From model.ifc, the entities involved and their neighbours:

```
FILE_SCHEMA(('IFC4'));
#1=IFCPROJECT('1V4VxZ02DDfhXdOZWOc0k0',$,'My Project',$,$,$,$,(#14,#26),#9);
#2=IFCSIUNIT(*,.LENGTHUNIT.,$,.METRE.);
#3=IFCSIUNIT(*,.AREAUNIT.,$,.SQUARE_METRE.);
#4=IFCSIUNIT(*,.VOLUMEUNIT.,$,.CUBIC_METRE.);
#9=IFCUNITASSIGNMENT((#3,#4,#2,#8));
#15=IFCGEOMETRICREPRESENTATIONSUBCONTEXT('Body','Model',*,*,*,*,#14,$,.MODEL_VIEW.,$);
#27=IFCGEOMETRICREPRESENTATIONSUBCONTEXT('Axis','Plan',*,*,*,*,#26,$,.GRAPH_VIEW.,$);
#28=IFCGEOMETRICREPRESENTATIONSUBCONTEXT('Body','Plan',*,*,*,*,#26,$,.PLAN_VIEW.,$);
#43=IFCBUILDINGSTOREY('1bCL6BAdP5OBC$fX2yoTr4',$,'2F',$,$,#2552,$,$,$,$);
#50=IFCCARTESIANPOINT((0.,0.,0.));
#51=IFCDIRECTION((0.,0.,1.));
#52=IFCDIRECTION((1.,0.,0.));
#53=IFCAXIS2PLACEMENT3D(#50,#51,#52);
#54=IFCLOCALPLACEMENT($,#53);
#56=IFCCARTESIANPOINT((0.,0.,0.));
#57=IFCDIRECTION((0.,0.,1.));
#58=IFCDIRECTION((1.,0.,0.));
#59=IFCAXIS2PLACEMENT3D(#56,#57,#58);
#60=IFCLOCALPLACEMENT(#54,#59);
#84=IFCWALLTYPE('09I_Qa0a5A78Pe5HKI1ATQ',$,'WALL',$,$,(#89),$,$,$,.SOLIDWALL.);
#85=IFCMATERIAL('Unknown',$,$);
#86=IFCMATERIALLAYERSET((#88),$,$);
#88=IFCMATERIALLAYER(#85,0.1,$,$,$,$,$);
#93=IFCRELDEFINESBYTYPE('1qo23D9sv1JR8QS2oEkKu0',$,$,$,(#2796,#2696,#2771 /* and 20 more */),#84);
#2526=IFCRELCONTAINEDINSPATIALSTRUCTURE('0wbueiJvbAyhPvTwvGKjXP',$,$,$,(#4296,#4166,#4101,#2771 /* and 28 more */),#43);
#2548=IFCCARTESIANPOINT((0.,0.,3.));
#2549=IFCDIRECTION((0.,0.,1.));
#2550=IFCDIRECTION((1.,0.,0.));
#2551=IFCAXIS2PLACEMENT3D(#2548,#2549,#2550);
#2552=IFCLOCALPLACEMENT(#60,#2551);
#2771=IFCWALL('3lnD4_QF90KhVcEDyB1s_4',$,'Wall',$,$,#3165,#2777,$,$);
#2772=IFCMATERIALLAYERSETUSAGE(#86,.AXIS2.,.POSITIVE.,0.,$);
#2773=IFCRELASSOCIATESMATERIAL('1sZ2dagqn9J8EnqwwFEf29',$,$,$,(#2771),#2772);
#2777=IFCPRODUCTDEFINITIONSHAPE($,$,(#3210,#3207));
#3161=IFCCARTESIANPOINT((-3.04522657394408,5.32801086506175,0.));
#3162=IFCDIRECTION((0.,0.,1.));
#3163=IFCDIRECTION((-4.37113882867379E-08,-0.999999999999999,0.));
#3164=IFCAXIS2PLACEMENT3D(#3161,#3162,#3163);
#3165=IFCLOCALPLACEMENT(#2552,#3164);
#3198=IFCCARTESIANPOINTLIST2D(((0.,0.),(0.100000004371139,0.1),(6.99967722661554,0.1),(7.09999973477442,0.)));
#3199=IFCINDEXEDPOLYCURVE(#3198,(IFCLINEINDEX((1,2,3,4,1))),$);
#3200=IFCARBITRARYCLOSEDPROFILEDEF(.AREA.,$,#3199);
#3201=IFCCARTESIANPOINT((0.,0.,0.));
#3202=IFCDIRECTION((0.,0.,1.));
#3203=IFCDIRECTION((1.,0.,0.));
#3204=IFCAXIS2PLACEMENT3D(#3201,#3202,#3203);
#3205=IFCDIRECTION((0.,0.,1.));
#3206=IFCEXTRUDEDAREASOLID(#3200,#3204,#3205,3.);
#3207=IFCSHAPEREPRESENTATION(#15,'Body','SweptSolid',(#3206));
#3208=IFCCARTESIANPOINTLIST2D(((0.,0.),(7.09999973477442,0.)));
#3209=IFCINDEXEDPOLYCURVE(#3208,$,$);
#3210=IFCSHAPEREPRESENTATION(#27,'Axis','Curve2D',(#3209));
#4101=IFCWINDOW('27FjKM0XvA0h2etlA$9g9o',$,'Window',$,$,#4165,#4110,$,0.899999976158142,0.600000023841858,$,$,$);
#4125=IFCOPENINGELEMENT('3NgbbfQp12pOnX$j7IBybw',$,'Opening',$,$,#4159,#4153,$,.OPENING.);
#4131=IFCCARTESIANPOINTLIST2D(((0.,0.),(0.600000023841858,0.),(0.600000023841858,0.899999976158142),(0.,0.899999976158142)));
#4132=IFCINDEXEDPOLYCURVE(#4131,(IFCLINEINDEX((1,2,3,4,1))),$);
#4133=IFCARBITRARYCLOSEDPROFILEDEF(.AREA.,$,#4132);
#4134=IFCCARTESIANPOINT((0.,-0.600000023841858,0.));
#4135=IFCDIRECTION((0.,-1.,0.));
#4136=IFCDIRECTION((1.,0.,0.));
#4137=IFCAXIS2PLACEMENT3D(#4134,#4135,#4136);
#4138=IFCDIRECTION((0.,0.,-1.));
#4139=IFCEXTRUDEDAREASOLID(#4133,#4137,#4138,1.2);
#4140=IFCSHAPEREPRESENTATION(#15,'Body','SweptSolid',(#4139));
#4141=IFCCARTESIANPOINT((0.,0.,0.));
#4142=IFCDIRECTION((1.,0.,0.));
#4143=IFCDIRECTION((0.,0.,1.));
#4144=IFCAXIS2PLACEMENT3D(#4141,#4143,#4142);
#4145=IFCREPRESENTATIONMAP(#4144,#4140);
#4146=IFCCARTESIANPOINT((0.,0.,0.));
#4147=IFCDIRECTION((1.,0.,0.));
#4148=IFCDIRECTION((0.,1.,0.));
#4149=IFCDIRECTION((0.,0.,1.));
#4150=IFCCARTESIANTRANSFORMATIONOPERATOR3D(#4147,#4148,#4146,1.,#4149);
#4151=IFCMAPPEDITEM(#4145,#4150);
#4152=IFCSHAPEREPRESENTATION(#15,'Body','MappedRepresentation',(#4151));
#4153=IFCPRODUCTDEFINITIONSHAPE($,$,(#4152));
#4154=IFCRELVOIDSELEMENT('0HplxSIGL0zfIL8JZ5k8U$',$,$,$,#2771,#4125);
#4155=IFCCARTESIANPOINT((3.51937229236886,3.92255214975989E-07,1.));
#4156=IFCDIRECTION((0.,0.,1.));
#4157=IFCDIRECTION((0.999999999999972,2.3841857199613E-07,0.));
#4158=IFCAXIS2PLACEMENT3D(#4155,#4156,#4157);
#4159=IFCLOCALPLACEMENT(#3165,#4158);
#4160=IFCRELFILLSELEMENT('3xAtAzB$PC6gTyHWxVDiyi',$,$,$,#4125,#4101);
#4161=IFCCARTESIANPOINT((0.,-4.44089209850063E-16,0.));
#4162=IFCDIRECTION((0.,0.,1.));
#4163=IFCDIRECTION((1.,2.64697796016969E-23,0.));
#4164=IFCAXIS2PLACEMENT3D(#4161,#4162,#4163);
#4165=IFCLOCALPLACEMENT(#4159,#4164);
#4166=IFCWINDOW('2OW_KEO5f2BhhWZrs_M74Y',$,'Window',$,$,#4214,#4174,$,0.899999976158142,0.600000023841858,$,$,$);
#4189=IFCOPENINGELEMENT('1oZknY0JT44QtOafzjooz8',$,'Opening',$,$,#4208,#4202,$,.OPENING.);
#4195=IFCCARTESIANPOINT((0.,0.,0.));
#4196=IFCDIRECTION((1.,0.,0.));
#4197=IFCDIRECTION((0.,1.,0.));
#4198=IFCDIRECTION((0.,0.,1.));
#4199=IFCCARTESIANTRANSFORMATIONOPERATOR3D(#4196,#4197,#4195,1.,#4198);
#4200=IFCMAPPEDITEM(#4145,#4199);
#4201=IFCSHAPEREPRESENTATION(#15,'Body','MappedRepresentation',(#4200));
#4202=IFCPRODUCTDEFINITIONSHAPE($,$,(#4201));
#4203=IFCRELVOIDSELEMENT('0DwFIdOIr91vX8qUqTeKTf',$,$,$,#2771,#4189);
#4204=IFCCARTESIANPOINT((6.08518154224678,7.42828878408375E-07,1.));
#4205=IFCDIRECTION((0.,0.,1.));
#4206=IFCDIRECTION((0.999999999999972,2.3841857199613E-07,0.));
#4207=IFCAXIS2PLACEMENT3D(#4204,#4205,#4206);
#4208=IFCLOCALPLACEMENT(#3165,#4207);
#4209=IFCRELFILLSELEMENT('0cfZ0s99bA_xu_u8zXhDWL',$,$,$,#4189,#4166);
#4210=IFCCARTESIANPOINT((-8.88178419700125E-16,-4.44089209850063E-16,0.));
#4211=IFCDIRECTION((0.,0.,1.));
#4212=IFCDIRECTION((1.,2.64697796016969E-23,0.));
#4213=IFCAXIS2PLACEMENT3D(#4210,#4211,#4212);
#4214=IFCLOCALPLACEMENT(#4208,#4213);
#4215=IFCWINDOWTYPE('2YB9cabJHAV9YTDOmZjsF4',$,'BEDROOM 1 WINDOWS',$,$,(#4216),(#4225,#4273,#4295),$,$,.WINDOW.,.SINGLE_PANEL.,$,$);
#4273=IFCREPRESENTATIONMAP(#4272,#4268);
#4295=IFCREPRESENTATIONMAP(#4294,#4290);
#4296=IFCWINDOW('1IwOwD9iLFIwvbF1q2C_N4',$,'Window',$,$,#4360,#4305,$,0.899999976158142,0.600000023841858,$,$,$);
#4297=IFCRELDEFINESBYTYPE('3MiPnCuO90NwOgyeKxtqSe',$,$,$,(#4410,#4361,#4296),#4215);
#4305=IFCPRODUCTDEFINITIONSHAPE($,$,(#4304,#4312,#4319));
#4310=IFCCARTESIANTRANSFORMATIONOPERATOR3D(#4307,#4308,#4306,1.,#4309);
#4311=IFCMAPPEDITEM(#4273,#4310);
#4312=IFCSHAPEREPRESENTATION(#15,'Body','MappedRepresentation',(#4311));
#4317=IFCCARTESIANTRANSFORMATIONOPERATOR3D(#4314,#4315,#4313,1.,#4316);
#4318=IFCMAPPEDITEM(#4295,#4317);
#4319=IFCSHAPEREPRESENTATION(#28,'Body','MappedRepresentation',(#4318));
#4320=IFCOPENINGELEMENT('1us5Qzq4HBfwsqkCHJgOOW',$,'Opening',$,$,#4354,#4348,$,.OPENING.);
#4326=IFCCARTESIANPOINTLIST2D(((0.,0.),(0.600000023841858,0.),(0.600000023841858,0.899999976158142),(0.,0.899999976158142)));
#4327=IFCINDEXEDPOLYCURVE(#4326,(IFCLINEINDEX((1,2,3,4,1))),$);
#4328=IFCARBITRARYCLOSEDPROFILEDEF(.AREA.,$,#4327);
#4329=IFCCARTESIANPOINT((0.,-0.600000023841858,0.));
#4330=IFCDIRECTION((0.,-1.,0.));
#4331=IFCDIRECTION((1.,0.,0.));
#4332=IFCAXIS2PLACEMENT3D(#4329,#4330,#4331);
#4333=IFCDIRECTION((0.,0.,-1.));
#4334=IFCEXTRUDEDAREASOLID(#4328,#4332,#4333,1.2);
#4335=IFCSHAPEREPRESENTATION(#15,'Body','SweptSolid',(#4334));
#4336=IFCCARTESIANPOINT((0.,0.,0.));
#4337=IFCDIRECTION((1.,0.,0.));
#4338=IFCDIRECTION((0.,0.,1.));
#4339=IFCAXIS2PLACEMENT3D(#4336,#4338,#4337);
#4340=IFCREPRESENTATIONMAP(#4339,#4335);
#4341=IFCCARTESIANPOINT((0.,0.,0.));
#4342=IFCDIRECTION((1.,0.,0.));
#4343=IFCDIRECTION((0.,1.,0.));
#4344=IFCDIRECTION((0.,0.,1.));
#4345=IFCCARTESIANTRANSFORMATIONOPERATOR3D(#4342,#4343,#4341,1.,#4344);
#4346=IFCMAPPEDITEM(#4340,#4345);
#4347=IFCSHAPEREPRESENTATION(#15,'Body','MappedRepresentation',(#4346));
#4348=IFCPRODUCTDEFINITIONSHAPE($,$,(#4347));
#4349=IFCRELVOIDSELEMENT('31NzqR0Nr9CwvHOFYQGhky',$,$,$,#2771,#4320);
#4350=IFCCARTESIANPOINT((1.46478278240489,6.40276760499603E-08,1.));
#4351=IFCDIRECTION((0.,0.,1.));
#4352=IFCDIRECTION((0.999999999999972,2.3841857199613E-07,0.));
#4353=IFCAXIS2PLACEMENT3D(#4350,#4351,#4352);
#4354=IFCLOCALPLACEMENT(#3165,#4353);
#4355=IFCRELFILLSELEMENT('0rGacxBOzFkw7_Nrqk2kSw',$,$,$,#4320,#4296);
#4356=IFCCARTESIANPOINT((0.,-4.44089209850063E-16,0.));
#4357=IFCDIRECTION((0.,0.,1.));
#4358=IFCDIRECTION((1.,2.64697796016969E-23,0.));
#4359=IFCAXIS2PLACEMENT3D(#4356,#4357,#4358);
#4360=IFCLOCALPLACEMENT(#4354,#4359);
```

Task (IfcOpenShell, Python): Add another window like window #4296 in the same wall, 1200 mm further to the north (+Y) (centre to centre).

```python
import ifcopenshell
import ifcopenshell.api.feature
import ifcopenshell.api.geometry
import ifcopenshell.api.root
import ifcopenshell.geom
import ifcopenshell.util.element
import ifcopenshell.util.placement
import ifcopenshell.util.shape
import ifcopenshell.util.unit

model = ifcopenshell.open("model.ifc")
unit_scale = ifcopenshell.util.unit.calculate_unit_scale(model)
settings = ifcopenshell.geom.settings()


def volume(element):
    """Net volume in cubic metres, openings subtracted."""
    shape = ifcopenshell.geom.create_shape(settings, element)
    return ifcopenshell.util.shape.get_volume(shape.geometry)


window = model.by_guid("1IwOwD9iLFIwvbF1q2C_N4")
opening = window.FillsVoids[0].RelatingOpeningElement
wall = opening.VoidsElements[0].RelatingBuildingElement
before = volume(wall)
shift = ifcopenshell.util.placement.get_local_placement(wall.ObjectPlacement)[:3, 0] * -1.2 / unit_scale

# copy_class copies the void relationship, type, container and properties, but no geometry.
new_opening = ifcopenshell.api.root.copy_class(model, product=opening)
new_opening.Representation = ifcopenshell.util.element.copy_deep(
    model, opening.Representation, exclude=["IfcGeometricRepresentationContext", "IfcRepresentationMap"]
)
new_window = ifcopenshell.api.root.copy_class(model, product=window)
new_window.Representation = ifcopenshell.util.element.copy_deep(
    model, window.Representation, exclude=["IfcGeometricRepresentationContext", "IfcRepresentationMap"]
)
ifcopenshell.api.feature.add_filling(model, opening=new_opening, element=new_window)

for old, new in ((opening, new_opening), (window, new_window)):
    matrix = ifcopenshell.util.placement.get_local_placement(old.ObjectPlacement)
    matrix[:3, 3] += shift
    ifcopenshell.api.geometry.edit_object_placement(model, product=new, matrix=matrix, is_si=False)

after = volume(wall)

print(f"wall volume {before:.3f} -> {after:.3f} m3")

model.write("model_updated.ifc")
```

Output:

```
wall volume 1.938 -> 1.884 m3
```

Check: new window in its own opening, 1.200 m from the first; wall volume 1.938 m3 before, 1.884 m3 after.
